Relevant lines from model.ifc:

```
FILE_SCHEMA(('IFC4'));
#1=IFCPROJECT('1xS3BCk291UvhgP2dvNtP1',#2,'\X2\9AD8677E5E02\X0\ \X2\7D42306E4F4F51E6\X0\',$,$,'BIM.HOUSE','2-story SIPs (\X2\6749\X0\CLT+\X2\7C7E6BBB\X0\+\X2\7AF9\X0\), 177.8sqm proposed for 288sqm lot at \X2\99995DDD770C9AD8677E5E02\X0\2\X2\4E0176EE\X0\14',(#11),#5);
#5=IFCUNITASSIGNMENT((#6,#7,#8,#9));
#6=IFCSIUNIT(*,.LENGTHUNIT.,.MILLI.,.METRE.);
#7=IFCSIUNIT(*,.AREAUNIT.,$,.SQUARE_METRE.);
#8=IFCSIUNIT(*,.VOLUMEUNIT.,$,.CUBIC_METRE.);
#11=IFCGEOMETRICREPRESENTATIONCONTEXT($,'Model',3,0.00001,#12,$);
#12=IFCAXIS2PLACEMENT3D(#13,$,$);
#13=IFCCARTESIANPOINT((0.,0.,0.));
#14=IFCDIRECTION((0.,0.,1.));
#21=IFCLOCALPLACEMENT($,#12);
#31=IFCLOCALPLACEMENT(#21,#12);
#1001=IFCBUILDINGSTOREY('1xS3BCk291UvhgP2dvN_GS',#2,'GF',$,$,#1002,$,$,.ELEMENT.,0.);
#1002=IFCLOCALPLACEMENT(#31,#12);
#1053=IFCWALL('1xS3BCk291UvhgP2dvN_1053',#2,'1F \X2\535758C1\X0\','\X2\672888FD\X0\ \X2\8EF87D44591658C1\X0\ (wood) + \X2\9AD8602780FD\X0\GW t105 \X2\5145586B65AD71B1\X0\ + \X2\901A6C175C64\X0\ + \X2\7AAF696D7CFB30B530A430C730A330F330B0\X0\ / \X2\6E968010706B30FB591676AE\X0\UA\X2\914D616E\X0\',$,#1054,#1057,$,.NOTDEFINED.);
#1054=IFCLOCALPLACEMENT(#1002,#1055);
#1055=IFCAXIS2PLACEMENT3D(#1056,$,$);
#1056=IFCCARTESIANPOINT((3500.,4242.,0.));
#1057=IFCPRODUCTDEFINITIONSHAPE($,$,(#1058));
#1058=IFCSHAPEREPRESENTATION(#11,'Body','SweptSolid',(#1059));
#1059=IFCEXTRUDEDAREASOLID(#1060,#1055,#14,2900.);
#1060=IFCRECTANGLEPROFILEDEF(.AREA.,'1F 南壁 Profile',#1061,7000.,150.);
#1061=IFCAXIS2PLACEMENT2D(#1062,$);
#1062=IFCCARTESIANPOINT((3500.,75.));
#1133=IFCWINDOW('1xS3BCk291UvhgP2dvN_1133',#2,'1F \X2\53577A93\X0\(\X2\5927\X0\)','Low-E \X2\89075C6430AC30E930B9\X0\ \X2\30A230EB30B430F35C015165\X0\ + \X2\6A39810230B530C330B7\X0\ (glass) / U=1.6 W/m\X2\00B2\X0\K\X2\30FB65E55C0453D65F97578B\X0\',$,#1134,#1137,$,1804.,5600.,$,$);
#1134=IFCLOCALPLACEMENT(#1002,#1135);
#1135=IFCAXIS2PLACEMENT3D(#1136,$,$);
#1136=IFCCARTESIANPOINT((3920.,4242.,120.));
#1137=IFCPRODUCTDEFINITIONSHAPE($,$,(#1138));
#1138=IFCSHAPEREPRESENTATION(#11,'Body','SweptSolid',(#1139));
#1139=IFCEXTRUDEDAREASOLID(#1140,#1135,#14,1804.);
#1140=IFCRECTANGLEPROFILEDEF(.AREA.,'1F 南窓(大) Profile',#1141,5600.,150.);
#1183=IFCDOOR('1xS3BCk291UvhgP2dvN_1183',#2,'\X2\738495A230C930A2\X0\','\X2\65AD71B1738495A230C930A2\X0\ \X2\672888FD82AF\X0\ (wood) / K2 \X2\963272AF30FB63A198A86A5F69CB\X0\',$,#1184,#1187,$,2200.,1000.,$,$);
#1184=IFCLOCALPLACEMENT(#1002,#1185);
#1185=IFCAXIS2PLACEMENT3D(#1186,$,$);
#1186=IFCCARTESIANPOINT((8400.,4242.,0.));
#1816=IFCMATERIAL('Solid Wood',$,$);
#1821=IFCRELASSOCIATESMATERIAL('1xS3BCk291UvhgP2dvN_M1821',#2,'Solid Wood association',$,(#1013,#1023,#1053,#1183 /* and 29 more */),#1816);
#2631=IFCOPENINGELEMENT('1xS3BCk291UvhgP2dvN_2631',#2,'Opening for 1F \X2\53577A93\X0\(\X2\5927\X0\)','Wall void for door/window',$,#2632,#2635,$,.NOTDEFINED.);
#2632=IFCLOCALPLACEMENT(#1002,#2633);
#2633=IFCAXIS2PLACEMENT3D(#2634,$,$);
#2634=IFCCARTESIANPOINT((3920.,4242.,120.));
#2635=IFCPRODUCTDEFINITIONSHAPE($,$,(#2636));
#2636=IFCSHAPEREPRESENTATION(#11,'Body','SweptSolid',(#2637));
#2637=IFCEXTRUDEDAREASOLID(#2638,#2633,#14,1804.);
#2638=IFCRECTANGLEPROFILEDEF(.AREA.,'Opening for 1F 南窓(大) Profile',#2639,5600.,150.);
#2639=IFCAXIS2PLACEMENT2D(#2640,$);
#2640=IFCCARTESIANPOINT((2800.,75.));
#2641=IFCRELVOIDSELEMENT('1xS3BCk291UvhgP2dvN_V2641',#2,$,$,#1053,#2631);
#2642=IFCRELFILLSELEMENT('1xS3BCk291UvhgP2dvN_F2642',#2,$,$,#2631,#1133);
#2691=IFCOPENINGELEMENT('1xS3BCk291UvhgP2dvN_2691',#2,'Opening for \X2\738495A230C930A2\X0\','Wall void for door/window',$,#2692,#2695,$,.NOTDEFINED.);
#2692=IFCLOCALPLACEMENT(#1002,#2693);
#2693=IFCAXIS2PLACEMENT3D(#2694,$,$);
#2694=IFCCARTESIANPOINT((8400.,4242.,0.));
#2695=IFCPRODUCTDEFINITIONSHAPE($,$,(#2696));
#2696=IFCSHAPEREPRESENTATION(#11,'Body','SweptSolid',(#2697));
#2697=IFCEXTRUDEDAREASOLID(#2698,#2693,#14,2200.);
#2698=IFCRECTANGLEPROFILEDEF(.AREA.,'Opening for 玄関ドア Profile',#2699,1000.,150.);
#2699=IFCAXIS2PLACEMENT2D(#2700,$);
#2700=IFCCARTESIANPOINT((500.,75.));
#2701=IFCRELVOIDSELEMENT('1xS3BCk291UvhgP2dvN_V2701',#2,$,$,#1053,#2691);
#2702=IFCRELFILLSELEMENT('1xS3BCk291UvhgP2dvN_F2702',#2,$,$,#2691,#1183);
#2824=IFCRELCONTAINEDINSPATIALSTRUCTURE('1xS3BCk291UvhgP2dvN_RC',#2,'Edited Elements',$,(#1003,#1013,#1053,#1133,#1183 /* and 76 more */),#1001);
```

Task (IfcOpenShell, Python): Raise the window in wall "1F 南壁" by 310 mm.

```python
import numpy as np
import ifcopenshell
import ifcopenshell.api.geometry
import ifcopenshell.util.placement
import ifcopenshell.util.unit

model = ifcopenshell.open("model.ifc")
unit_scale = ifcopenshell.util.unit.calculate_unit_scale(model)

window = model.by_guid("1xS3BCk291UvhgP2dvN_1133")
opening = window.FillsVoids[0].RelatingOpeningElement
dz = 0.31 / unit_scale

shift = np.array([0.0, 0.0, dz])
# The window is not placed relative to its opening, so move both.
for product in (opening, window):
    matrix = ifcopenshell.util.placement.get_local_placement(product.ObjectPlacement)
    matrix[:3, 3] += shift
    ifcopenshell.api.geometry.edit_object_placement(model, product=product, matrix=matrix, is_si=False)

print(f"moved by {dz * unit_scale:+.3f} m")

model.write("model_edited.ifc")
```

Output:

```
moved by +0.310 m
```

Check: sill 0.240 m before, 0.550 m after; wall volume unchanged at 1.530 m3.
